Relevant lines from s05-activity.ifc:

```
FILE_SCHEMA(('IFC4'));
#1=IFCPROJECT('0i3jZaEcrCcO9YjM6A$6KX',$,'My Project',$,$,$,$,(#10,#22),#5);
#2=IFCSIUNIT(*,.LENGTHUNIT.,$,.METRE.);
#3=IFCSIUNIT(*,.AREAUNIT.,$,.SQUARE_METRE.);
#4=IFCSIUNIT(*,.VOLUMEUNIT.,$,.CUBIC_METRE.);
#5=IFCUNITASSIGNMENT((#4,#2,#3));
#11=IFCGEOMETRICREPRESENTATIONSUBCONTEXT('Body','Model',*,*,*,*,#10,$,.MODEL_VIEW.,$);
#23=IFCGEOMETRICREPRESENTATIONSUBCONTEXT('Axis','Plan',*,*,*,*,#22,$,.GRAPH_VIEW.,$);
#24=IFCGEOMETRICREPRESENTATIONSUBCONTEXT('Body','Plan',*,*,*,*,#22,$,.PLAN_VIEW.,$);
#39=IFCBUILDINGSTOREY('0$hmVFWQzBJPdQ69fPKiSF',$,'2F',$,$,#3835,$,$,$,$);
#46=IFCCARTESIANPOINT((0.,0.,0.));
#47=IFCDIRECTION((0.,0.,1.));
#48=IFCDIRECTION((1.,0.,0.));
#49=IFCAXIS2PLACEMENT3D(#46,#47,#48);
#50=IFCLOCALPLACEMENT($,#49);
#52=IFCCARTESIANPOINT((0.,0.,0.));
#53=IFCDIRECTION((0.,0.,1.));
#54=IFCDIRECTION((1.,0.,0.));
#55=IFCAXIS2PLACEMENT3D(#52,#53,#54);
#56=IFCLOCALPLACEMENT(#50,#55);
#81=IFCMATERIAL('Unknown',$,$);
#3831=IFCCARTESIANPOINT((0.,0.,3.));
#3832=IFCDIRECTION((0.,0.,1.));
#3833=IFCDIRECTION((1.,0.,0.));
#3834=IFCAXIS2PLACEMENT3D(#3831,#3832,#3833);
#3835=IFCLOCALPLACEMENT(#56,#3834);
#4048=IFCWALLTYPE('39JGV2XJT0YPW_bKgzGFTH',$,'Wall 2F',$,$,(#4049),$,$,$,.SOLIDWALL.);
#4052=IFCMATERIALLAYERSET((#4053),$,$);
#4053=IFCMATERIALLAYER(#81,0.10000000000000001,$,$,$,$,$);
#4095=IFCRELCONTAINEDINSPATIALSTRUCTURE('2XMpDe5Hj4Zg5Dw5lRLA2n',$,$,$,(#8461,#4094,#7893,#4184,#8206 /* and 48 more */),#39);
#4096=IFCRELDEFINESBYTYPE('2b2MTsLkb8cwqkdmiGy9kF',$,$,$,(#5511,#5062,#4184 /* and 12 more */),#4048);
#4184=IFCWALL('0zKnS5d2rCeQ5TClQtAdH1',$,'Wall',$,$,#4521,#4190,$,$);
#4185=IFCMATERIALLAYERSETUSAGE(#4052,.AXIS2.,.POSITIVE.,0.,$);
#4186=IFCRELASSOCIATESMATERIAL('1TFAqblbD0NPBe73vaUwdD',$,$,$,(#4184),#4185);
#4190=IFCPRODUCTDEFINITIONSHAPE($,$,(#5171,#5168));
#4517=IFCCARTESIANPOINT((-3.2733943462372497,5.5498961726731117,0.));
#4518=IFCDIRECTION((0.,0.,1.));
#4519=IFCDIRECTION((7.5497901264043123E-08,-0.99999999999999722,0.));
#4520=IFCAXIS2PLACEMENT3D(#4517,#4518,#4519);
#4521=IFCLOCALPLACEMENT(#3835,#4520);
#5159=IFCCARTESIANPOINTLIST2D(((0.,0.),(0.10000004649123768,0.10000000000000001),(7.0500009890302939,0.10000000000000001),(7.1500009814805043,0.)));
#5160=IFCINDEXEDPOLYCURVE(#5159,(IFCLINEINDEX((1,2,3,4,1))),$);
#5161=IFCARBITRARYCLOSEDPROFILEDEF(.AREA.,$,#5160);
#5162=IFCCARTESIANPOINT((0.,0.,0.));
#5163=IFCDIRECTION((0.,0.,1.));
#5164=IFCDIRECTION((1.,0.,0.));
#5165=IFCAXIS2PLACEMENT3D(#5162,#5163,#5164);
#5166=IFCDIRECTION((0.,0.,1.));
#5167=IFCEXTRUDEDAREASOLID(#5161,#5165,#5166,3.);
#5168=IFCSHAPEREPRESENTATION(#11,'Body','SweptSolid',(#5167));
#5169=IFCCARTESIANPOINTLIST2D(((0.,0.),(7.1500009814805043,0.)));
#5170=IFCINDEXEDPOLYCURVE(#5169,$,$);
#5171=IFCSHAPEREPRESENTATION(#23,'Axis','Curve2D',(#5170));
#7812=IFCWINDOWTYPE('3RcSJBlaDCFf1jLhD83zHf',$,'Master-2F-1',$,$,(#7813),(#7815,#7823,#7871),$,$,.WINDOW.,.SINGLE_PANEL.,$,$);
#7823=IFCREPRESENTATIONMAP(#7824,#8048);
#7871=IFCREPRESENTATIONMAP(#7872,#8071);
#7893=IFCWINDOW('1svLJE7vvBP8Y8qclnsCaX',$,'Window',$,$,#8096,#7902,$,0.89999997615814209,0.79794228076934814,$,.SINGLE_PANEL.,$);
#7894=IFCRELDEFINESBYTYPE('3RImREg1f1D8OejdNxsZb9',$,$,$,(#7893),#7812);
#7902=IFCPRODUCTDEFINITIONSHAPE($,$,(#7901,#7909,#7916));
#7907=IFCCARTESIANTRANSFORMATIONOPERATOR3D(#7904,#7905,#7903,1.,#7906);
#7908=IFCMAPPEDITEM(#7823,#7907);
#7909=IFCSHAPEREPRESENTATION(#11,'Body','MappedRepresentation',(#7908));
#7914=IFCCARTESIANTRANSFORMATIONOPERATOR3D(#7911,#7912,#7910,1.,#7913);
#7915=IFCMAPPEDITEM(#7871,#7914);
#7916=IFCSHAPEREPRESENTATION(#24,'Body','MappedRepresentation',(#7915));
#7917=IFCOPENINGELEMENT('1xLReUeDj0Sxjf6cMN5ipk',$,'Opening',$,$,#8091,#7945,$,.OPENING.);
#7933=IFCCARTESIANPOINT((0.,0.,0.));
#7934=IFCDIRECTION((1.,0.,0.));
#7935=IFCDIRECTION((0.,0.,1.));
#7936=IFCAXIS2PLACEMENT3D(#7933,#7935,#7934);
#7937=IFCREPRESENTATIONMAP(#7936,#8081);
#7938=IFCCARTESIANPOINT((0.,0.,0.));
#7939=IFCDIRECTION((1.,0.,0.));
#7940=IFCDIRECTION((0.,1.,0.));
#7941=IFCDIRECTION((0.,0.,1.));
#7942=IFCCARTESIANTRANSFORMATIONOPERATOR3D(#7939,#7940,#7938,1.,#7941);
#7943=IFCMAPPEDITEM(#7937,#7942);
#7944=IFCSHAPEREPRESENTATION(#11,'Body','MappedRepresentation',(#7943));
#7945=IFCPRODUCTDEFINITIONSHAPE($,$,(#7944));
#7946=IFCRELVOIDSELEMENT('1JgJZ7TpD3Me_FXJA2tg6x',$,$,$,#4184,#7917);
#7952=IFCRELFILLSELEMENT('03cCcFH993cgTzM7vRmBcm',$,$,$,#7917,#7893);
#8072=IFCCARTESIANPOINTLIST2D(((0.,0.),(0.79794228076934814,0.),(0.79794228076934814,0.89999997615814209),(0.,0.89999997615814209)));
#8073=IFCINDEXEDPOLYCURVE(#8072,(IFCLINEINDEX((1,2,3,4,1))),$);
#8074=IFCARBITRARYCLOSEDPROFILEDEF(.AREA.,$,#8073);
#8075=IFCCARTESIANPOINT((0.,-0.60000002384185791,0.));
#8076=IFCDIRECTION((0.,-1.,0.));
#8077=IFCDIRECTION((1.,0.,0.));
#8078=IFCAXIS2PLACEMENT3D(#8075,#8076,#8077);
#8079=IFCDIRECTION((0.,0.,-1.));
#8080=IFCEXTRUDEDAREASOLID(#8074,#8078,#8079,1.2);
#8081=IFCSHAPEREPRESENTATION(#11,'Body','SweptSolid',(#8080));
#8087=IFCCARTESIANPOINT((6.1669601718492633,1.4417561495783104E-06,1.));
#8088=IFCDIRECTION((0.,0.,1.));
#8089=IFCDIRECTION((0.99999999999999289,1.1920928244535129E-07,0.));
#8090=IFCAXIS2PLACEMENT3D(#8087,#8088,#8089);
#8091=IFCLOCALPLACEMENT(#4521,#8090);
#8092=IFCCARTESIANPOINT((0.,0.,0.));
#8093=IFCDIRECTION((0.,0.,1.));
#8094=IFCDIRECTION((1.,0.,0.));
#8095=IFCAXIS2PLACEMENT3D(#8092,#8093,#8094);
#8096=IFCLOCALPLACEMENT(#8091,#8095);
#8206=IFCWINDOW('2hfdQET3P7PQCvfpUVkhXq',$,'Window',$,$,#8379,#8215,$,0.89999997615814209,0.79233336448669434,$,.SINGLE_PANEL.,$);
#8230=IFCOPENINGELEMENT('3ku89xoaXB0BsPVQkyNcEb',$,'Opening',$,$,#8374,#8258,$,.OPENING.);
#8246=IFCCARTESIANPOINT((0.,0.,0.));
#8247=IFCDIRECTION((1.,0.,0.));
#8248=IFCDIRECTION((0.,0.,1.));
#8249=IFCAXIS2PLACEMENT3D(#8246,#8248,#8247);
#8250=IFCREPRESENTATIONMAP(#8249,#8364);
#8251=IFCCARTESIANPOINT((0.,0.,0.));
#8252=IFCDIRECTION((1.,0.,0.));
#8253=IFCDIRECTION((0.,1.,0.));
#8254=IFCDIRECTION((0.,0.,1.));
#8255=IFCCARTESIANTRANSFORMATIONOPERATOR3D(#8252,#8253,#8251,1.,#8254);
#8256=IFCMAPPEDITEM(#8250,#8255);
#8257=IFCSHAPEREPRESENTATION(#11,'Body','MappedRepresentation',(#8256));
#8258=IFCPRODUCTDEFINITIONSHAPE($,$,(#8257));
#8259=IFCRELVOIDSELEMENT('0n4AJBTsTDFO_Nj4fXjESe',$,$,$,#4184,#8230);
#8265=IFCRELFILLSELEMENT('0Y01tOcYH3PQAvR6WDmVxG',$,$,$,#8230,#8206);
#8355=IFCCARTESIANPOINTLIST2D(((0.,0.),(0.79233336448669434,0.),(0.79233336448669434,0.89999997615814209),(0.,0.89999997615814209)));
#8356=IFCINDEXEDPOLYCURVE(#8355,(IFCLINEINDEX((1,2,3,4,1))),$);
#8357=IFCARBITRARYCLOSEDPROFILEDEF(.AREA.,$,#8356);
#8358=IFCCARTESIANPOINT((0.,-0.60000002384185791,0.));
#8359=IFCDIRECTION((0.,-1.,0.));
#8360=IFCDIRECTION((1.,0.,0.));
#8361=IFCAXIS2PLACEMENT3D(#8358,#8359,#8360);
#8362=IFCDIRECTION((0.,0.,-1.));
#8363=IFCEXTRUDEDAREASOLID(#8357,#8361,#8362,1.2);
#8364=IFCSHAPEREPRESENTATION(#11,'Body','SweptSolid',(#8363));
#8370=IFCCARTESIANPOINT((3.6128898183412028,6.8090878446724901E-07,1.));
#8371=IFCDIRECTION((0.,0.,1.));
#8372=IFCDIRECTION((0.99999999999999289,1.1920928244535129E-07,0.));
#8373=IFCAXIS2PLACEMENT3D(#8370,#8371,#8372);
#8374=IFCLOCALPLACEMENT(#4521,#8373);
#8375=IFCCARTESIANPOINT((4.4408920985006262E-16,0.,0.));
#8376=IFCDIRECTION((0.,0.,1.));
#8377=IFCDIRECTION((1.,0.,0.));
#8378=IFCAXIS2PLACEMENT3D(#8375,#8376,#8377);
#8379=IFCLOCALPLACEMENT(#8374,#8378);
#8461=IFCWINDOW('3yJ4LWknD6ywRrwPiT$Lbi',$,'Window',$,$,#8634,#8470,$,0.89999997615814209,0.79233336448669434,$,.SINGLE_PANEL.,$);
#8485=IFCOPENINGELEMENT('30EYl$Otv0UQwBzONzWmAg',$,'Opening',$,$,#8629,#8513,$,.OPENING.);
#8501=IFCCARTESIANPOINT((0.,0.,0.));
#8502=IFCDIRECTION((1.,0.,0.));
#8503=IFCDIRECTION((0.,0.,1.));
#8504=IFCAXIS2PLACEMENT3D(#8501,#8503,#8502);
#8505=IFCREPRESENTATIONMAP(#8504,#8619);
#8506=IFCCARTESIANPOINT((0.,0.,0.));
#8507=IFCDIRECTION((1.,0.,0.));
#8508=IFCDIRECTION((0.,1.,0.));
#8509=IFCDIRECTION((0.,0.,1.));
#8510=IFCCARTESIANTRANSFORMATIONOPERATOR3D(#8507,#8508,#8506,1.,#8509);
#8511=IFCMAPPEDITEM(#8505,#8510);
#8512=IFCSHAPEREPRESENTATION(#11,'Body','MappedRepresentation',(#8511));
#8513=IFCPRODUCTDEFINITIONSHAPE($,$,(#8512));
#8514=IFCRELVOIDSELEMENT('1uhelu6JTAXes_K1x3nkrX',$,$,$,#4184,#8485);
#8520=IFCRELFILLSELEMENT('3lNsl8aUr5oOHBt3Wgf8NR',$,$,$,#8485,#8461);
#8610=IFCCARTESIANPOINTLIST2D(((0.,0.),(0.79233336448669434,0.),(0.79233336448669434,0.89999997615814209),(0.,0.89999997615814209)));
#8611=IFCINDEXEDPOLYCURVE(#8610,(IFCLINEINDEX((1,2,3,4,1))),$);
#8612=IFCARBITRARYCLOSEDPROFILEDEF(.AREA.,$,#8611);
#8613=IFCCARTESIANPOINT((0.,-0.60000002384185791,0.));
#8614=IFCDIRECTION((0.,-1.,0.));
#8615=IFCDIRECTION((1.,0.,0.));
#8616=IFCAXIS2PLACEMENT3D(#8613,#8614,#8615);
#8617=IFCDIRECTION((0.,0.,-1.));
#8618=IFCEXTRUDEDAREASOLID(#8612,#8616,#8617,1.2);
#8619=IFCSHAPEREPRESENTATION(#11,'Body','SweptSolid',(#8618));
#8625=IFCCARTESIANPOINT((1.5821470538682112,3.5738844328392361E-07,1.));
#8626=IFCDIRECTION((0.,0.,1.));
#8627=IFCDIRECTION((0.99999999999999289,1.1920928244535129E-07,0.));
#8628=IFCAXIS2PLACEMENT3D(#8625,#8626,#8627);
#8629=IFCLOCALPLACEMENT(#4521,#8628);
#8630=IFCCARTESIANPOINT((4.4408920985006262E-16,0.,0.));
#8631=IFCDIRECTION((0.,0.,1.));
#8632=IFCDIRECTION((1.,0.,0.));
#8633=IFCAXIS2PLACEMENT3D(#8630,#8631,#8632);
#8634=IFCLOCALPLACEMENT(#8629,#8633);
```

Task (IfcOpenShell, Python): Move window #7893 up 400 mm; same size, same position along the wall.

```python
import numpy as np
import ifcopenshell
import ifcopenshell.api.geometry
import ifcopenshell.util.placement
import ifcopenshell.util.unit

model = ifcopenshell.open("s05-activity.ifc")
unit_scale = ifcopenshell.util.unit.calculate_unit_scale(model)

window = model.by_guid("1svLJE7vvBP8Y8qclnsCaX")
opening = window.FillsVoids[0].RelatingOpeningElement
dz = 0.4 / unit_scale

shift = np.array([0.0, 0.0, dz])
# The window is placed relative to its opening, so it follows when the opening moves.
matrix = ifcopenshell.util.placement.get_local_placement(opening.ObjectPlacement)
matrix[:3, 3] += shift
ifcopenshell.api.geometry.edit_object_placement(
    model, product=opening, matrix=matrix, is_si=False, should_transform_children=True
)

print(f"moved by {dz * unit_scale:+.3f} m")

model.write("s05-activity-out.ifc")
```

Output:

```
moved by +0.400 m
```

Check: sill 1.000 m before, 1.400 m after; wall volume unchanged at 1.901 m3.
